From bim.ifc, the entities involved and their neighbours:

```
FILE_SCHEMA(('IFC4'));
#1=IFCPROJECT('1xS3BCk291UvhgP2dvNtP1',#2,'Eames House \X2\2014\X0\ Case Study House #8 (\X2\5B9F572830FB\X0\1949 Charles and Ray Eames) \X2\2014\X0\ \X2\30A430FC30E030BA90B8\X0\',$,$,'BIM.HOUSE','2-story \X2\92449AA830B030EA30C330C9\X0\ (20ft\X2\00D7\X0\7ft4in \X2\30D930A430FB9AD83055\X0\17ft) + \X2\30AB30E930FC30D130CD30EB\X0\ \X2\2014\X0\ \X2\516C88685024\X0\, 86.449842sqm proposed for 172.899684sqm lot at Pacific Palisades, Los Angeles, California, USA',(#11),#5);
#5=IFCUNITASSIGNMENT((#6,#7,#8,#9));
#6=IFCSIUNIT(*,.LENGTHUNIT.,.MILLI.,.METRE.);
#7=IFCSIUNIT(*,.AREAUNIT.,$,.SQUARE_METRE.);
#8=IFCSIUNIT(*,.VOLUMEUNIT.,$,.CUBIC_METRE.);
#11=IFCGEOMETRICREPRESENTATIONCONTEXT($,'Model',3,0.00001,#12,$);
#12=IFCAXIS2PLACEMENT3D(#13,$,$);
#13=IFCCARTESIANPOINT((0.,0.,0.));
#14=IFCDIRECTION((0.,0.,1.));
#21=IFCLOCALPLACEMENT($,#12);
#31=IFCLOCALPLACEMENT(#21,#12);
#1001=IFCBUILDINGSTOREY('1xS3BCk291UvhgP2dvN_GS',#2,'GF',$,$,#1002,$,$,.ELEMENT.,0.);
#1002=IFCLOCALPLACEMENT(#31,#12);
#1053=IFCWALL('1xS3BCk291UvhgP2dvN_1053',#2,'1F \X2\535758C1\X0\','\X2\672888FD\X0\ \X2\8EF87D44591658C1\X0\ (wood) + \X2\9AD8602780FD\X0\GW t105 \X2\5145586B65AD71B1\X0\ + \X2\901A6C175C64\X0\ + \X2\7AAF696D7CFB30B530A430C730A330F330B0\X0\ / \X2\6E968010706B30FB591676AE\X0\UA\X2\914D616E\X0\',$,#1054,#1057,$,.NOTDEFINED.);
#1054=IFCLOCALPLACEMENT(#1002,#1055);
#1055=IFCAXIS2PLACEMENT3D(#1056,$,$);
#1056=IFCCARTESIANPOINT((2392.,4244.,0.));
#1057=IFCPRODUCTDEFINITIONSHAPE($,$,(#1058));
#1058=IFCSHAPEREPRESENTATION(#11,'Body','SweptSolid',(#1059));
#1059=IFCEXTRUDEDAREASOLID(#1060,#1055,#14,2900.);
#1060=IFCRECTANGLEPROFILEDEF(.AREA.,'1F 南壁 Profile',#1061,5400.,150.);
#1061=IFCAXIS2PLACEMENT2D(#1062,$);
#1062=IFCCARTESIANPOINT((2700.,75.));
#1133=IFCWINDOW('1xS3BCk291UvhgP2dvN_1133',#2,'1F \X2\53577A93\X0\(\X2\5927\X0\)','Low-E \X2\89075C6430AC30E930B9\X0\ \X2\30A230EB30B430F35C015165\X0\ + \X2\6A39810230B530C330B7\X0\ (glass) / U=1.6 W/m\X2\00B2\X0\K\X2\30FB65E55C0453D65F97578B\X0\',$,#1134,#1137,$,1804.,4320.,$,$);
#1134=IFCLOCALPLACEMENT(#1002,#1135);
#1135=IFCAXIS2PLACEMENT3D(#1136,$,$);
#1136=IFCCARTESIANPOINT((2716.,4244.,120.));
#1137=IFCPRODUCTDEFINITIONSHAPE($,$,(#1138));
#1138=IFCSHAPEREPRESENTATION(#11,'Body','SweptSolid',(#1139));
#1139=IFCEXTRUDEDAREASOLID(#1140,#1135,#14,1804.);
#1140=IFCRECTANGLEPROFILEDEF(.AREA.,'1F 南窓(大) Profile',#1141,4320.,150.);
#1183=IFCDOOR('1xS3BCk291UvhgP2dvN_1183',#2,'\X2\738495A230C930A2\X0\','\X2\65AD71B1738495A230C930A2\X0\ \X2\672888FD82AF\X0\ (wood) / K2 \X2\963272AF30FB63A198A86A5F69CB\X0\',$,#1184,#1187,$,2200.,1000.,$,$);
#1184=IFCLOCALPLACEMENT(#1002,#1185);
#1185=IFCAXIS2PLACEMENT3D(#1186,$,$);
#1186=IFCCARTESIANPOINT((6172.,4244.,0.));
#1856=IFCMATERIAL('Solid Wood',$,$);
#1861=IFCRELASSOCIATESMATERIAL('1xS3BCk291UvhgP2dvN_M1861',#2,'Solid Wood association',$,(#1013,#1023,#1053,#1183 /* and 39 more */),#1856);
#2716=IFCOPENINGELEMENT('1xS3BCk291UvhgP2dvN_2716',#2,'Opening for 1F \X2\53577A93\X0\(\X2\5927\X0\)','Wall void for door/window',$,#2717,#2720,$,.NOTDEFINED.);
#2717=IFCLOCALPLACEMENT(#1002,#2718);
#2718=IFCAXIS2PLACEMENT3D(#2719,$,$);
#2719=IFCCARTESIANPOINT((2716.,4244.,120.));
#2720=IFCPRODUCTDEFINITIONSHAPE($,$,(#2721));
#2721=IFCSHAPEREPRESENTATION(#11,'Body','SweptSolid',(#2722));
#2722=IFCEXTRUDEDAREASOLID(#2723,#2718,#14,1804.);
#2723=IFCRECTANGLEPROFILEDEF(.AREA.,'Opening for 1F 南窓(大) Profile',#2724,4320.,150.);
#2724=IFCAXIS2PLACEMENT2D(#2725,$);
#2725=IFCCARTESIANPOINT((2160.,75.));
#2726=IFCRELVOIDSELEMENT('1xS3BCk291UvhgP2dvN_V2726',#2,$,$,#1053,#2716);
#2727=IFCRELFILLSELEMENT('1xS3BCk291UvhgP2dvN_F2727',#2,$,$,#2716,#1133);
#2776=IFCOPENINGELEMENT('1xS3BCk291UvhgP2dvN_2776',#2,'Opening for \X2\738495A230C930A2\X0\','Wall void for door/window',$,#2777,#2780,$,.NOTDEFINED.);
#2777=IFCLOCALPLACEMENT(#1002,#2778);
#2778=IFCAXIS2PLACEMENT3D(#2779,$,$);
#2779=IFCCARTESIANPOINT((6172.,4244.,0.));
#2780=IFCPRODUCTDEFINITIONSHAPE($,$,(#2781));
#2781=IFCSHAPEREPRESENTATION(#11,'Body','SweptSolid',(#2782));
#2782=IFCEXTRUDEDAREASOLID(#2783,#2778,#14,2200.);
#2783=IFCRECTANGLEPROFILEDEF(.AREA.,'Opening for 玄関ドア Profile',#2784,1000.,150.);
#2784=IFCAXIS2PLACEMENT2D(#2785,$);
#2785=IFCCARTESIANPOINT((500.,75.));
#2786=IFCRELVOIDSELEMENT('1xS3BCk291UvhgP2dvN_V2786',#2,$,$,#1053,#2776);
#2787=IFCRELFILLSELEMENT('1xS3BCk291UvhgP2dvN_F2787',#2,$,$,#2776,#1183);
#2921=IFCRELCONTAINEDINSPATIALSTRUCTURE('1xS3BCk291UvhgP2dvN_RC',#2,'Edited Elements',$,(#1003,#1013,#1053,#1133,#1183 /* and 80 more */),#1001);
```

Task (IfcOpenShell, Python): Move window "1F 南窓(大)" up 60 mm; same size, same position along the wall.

```python
import numpy as np
import ifcopenshell
import ifcopenshell.api.geometry
import ifcopenshell.util.placement
import ifcopenshell.util.unit

model = ifcopenshell.open("bim.ifc")
unit_scale = ifcopenshell.util.unit.calculate_unit_scale(model)

window = model.by_guid("1xS3BCk291UvhgP2dvN_1133")
opening = window.FillsVoids[0].RelatingOpeningElement
dz = 60.0

shift = np.array([0.0, 0.0, dz])
# The window is not placed relative to its opening, so move both.
for product in (opening, window):
    matrix = ifcopenshell.util.placement.get_local_placement(product.ObjectPlacement)
    matrix[:3, 3] += shift
    ifcopenshell.api.geometry.edit_object_placement(model, product=product, matrix=matrix, is_si=False)

print(f"moved by {dz * unit_scale:+.3f} m")

model.write("bim-out.ifc")
```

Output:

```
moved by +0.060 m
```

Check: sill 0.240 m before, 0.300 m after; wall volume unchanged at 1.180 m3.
